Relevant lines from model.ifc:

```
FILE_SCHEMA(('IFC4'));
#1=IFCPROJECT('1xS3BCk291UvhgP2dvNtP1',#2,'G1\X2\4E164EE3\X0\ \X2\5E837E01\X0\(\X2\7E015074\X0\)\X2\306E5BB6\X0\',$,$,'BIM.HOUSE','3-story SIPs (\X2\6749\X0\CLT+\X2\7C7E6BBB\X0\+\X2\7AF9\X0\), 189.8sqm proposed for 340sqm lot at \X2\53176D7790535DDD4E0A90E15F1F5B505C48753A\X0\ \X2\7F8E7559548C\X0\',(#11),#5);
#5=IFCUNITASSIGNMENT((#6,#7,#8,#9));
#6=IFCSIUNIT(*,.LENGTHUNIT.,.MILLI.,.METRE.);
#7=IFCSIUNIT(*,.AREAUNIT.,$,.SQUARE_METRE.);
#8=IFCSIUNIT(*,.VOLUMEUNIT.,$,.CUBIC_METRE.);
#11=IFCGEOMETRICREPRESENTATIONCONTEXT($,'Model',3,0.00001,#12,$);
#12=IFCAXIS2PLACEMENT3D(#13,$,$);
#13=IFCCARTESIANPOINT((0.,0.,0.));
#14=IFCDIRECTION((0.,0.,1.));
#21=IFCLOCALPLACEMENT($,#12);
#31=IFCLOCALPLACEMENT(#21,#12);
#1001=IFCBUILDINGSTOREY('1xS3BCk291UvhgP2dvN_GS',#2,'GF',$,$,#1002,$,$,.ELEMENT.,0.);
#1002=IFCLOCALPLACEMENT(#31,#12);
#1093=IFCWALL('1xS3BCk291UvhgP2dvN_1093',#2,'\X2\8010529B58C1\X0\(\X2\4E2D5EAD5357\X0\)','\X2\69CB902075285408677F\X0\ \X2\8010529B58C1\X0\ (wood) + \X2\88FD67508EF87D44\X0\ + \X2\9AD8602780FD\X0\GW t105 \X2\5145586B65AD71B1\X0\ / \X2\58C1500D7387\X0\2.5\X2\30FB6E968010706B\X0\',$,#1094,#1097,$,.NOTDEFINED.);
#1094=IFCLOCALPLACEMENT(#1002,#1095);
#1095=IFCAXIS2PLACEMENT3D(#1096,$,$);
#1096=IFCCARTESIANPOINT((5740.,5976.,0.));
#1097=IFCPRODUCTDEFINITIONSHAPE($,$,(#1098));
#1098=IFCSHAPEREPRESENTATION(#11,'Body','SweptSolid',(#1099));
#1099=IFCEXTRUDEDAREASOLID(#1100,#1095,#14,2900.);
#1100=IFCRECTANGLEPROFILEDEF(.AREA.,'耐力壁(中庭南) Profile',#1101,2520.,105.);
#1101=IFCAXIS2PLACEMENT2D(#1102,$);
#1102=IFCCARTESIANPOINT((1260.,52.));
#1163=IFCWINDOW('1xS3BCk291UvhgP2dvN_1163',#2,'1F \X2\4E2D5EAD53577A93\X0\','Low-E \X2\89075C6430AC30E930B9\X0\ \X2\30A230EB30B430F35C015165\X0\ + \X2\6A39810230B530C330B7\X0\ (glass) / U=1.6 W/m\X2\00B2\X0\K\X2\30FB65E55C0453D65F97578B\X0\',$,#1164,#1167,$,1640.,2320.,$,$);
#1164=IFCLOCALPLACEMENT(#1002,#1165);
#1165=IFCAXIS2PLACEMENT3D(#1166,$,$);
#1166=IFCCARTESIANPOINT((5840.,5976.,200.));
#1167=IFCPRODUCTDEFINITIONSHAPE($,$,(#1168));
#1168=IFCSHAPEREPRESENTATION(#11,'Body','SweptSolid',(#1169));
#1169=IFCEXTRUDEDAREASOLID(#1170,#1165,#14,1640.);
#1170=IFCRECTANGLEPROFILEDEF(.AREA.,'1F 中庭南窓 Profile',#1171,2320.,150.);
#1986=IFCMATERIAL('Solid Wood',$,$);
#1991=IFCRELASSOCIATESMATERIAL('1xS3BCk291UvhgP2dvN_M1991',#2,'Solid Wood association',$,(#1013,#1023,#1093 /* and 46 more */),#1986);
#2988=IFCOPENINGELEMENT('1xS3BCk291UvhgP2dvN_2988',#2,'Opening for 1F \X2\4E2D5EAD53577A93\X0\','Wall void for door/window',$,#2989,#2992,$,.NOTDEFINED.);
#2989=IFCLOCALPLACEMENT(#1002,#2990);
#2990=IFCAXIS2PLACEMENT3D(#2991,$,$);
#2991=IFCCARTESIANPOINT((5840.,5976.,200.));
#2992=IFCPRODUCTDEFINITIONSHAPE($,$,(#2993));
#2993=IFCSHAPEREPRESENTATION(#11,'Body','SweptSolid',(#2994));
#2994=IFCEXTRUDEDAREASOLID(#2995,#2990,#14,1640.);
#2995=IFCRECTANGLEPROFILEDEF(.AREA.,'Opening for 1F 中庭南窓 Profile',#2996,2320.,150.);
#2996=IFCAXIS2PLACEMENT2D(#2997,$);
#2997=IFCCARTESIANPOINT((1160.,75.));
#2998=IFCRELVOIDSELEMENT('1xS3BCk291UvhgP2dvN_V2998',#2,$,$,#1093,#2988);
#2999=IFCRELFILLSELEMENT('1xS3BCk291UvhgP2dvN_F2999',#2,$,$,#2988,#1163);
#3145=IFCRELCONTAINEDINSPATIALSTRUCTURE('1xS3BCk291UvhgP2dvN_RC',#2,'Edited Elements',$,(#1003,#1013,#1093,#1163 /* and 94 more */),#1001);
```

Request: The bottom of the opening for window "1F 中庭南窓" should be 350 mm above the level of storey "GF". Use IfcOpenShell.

```python
import numpy as np
import ifcopenshell
import ifcopenshell.api.geometry
import ifcopenshell.geom
import ifcopenshell.util.element
import ifcopenshell.util.placement
import ifcopenshell.util.shape
import ifcopenshell.util.unit

model = ifcopenshell.open("model.ifc")
unit_scale = ifcopenshell.util.unit.calculate_unit_scale(model)

window = model.by_guid("1xS3BCk291UvhgP2dvN_1163")
opening = window.FillsVoids[0].RelatingOpeningElement
storey = ifcopenshell.util.element.get_container(window, ifc_class="IfcBuildingStorey")
level = ifcopenshell.util.placement.get_local_placement(storey.ObjectPlacement)[2, 3]

# The opening's origin need not be at the sill, so measure its lowest point.
shape = ifcopenshell.geom.create_shape(ifcopenshell.geom.settings(), opening)
bottom = ifcopenshell.util.shape.get_shape_bottom_elevation(shape, shape.geometry) / unit_scale
dz = level + 0.35 / unit_scale - bottom

shift = np.array([0.0, 0.0, dz])
# The window is not placed relative to its opening, so move both.
for product in (opening, window):
    matrix = ifcopenshell.util.placement.get_local_placement(product.ObjectPlacement)
    matrix[:3, 3] += shift
    ifcopenshell.api.geometry.edit_object_placement(model, product=product, matrix=matrix, is_si=False)

print(f"moved by {dz * unit_scale:+.3f} m")

model.write("model_v2.ifc")
```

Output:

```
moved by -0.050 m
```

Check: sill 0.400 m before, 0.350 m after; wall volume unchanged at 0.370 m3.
